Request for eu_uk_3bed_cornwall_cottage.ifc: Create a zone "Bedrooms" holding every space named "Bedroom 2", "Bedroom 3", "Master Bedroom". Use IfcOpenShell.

First a look at what the model holds.

```python
import ifcopenshell

model = ifcopenshell.open("eu_uk_3bed_cornwall_cottage.ifc")
print(model.schema)
seen = {}
for space in model.by_type("IfcSpace"):
    seen[space.LongName] = seen.get(space.LongName, 0) + 1
for name, count in sorted(seen.items(), key=str):
    print(count, "x", name)
print("zones:", [z.Name for z in model.by_type("IfcZone")][:20])
```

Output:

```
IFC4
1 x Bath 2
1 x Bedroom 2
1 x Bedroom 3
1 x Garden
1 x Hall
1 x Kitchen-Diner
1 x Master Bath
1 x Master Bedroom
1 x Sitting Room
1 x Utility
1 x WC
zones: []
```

```python
import ifcopenshell
import ifcopenshell.api.group
import ifcopenshell.api.root

model = ifcopenshell.open("eu_uk_3bed_cornwall_cottage.ifc")

names = {"Bedroom 2", "Bedroom 3", "Master Bedroom"}
spaces = [s for s in model.by_type("IfcSpace") if s.LongName in names]

zone = ifcopenshell.api.root.create_entity(model, ifc_class="IfcZone", name="Bedrooms")
ifcopenshell.api.group.assign_group(model, products=spaces, group=zone)
print(len(spaces), "spaces in", zone.Name)

model.write("eu_uk_3bed_cornwall_cottage-out.ifc")
```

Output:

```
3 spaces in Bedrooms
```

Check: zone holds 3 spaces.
